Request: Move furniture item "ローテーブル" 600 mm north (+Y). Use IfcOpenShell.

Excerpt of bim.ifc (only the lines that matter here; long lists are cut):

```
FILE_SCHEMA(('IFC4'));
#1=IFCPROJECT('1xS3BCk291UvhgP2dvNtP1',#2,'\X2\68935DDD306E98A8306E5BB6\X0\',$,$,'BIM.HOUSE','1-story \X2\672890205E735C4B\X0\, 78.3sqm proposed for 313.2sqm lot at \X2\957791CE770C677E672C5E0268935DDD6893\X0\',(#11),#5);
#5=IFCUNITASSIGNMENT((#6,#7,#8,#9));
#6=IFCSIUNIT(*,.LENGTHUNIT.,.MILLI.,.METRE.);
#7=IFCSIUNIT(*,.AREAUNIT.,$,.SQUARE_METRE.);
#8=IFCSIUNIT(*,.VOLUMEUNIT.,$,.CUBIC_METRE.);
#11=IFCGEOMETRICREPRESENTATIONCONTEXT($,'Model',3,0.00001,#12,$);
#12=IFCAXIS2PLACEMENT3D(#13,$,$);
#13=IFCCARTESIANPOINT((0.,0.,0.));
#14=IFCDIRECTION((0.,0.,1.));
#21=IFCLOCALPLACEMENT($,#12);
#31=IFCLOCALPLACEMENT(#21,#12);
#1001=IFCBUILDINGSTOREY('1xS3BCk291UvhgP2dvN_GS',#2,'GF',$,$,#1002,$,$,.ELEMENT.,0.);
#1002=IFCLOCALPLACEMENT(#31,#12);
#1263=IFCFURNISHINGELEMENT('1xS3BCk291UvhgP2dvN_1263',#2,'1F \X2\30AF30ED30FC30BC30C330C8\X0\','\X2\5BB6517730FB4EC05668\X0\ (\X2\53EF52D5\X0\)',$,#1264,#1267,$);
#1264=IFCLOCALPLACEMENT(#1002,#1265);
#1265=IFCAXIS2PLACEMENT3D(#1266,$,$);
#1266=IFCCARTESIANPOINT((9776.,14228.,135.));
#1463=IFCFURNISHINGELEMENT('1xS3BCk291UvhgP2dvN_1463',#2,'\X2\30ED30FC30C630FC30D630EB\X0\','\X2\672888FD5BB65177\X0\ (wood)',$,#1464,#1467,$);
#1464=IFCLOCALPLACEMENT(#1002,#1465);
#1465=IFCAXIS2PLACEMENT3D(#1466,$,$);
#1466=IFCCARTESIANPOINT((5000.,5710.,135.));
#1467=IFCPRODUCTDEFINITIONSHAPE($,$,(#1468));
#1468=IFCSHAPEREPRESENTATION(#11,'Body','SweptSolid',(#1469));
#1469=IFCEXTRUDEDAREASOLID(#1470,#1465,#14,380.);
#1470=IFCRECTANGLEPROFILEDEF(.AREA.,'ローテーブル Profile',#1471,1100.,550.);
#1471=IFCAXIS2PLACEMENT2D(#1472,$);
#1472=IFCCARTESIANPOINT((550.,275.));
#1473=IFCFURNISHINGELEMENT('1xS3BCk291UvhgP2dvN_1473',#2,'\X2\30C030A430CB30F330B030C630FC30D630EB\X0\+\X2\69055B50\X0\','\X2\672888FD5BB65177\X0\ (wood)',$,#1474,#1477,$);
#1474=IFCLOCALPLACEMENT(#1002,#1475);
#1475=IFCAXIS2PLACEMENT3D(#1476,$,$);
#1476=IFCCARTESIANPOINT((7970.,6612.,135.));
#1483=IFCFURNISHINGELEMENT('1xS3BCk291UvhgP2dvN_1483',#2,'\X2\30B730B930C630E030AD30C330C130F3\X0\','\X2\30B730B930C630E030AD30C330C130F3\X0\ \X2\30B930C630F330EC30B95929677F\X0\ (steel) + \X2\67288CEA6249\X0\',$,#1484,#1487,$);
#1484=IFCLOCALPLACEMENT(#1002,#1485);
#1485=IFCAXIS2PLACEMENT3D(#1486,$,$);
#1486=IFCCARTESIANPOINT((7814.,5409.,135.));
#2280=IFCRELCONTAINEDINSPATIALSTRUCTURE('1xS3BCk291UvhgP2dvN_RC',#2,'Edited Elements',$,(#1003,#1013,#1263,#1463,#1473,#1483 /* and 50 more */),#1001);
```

```python
import ifcopenshell
import ifcopenshell.api.geometry
import ifcopenshell.util.placement

model = ifcopenshell.open("bim.ifc")

item = model.by_id(1463)
matrix = ifcopenshell.util.placement.get_local_placement(item.ObjectPlacement)
matrix[1, 3] += 600.0
ifcopenshell.api.geometry.edit_object_placement(model, product=item, matrix=matrix, is_si=False)

print(ifcopenshell.util.placement.get_local_placement(item.ObjectPlacement).round(3) + 0.0)

model.write("bim_rev.ifc")
```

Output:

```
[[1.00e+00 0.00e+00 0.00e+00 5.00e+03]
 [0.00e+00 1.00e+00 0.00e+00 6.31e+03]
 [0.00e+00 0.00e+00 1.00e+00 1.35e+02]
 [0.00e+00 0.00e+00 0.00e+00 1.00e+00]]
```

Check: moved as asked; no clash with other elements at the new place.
